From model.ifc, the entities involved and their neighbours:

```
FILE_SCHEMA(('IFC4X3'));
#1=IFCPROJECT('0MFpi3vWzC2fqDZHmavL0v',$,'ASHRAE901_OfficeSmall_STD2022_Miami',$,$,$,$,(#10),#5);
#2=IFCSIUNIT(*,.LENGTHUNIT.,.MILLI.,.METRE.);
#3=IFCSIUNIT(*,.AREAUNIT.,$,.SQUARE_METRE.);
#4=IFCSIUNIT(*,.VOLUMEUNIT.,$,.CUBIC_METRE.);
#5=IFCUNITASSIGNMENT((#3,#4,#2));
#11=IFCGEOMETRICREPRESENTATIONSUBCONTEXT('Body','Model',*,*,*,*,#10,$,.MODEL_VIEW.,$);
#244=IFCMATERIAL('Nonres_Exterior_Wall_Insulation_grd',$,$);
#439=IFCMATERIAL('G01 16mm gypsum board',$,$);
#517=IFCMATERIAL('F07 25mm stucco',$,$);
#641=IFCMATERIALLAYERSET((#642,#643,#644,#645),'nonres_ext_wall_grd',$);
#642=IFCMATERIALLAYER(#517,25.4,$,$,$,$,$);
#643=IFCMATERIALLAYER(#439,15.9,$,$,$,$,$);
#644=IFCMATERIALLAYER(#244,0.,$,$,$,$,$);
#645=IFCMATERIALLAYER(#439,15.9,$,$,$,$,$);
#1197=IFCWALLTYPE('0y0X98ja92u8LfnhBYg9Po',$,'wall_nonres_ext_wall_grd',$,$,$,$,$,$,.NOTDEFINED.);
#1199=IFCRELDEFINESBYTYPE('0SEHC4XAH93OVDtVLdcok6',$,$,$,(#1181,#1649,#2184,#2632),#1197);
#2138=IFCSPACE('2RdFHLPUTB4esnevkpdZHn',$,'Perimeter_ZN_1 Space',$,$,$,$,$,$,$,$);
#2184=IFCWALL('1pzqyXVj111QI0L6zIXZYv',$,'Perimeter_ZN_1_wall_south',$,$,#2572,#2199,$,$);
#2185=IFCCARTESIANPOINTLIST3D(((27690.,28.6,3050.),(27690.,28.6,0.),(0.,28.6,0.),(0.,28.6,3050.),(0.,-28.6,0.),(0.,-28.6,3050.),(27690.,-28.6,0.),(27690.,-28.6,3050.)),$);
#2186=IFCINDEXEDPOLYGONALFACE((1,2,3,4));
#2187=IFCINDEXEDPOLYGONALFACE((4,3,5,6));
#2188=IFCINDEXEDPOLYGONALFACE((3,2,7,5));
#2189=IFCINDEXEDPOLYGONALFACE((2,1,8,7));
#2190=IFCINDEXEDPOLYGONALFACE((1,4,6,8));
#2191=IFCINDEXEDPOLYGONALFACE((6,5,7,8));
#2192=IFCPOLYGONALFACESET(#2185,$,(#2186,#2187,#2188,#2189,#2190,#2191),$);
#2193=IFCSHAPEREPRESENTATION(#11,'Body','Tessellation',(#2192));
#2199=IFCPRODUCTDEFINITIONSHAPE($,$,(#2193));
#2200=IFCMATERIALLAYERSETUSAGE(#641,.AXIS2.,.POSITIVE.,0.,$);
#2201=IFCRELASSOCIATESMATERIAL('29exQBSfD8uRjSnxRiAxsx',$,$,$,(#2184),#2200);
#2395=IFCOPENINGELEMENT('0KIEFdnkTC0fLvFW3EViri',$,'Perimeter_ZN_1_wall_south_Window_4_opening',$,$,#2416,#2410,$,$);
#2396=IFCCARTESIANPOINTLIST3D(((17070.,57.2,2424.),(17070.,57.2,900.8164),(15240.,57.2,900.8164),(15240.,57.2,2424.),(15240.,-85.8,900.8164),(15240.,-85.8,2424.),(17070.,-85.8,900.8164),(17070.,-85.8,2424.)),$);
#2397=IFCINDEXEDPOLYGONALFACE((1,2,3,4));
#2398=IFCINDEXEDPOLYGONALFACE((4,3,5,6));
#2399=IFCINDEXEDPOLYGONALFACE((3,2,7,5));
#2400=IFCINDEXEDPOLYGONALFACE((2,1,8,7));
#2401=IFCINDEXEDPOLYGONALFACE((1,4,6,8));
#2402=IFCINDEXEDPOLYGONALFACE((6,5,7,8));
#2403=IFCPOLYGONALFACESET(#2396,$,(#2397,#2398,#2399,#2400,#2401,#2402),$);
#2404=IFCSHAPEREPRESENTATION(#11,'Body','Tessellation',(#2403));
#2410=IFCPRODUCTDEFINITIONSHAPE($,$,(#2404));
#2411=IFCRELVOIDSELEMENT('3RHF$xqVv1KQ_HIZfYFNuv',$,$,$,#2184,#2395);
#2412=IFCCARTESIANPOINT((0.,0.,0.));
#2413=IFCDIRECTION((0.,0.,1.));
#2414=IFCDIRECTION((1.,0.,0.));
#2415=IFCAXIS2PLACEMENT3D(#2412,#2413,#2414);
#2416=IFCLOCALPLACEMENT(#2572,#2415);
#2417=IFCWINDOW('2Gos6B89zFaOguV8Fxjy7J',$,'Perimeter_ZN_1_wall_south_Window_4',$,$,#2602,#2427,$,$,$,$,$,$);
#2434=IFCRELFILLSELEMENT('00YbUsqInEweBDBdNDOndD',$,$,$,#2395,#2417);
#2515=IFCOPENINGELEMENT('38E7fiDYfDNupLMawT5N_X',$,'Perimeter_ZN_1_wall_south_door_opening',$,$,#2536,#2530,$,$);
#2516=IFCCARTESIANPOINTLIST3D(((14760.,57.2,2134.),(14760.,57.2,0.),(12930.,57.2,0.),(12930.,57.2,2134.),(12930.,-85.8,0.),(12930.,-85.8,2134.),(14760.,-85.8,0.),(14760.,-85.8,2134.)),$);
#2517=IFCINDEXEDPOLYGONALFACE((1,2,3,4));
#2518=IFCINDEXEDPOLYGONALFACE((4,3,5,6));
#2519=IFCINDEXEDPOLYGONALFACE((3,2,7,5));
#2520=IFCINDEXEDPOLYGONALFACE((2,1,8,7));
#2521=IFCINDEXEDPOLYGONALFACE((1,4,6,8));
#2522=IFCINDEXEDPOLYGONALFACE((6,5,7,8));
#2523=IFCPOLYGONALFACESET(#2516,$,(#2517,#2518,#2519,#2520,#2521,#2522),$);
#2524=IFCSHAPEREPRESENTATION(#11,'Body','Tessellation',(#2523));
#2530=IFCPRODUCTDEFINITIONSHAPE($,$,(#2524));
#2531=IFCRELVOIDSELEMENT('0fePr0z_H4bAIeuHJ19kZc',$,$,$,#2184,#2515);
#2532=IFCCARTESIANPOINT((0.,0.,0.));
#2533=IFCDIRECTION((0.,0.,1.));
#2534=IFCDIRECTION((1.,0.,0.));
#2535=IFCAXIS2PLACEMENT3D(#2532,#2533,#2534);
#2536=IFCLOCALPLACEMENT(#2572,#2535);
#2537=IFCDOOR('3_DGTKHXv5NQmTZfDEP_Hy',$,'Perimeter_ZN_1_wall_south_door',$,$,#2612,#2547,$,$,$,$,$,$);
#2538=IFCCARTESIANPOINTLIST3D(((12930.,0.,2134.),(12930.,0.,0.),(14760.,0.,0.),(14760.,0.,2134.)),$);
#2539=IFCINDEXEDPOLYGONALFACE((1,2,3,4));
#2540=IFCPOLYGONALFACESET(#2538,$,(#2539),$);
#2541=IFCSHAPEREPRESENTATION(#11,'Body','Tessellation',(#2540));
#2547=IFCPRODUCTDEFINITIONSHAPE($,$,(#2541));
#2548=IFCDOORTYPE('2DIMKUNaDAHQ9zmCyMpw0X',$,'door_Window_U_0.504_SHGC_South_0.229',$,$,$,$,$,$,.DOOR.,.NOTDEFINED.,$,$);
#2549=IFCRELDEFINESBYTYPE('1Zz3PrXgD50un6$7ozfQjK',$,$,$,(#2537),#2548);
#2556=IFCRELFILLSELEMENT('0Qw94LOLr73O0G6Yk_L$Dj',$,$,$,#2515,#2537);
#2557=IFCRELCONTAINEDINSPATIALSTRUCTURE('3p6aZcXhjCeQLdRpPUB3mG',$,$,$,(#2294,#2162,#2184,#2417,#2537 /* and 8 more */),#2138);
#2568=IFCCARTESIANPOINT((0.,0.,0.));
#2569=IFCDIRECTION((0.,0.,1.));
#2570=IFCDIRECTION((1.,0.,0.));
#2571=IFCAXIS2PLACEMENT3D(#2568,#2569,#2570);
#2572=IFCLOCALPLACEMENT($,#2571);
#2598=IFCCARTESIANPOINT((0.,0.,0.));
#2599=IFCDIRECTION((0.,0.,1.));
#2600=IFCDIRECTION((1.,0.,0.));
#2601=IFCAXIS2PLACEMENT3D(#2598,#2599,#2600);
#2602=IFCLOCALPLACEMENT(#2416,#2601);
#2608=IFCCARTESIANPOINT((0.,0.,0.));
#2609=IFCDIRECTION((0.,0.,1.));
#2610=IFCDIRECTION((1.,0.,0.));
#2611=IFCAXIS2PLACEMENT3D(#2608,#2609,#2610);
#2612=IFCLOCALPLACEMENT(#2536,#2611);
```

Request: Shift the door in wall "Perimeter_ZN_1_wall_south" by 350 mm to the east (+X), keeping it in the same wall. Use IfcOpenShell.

```python
import ifcopenshell
import ifcopenshell.api.geometry
import ifcopenshell.util.placement
import ifcopenshell.util.unit

model = ifcopenshell.open("model.ifc")
unit_scale = ifcopenshell.util.unit.calculate_unit_scale(model)

door = model.by_id(2537)
opening = door.FillsVoids[0].RelatingOpeningElement
wall = opening.VoidsElements[0].RelatingBuildingElement

wall_matrix = ifcopenshell.util.placement.get_local_placement(wall.ObjectPlacement)
shift = wall_matrix[:3, 0] * 0.35 / unit_scale
before = ifcopenshell.util.placement.get_local_placement(door.ObjectPlacement)[:3, 3].copy()

# The door is placed relative to its opening, so it follows when the opening moves.
matrix = ifcopenshell.util.placement.get_local_placement(opening.ObjectPlacement)
matrix[:3, 3] += shift
ifcopenshell.api.geometry.edit_object_placement(
    model, product=opening, matrix=matrix, is_si=False, should_transform_children=True
)

after = ifcopenshell.util.placement.get_local_placement(door.ObjectPlacement)[:3, 3]
print("door moved by", (after - before).round(3) + 0.0)

model.write("model_v2.ifc")
```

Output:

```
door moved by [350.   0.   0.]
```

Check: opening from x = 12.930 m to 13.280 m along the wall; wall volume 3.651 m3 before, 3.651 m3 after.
